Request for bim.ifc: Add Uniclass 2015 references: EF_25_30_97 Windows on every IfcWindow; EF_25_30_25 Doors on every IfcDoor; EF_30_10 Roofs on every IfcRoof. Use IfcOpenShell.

First a look at what the model holds.

```python
import ifcopenshell

model = ifcopenshell.open("bim.ifc")
print(model.schema)
print("classifications:", [c.Name for c in model.by_type("IfcClassification")])
for ifc_class in ("IfcDoor", "IfcRoof", "IfcStair", "IfcWall", "IfcWindow"):
    print(ifc_class, len(model.by_type(ifc_class)))
```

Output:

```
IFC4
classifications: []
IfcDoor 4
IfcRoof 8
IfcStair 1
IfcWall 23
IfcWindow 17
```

```python
import ifcopenshell
import ifcopenshell.api.classification

model = ifcopenshell.open("bim.ifc")

system = ifcopenshell.api.classification.add_classification(model, classification="Uniclass 2015")

codes = {
    "IfcWindow": ("EF_25_30_97", "Windows"),
    "IfcDoor": ("EF_25_30_25", "Doors"),
    "IfcRoof": ("EF_30_10", "Roofs"),
}
for ifc_class, (code, name) in codes.items():
    products = model.by_type(ifc_class)
    ifcopenshell.api.classification.add_reference(
        model, products=products, classification=system, identification=code, name=name
    )
    print(code, len(products))

model.write("bim-out.ifc")
```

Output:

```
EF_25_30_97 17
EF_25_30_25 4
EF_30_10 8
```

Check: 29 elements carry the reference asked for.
